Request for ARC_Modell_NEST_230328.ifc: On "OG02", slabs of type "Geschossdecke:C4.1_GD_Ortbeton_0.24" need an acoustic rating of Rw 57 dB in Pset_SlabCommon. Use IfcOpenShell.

First a look at what the model holds.

```python
import ifcopenshell
import ifcopenshell.util.element

model = ifcopenshell.open("ARC_Modell_NEST_230328.ifc")
print(model.schema)
storey = next(s for s in model.by_type("IfcBuildingStorey") if s.Name == "OG02")
slabs = [e for e in ifcopenshell.util.element.get_decomposition(storey) if e.is_a("IfcSlab")]
seen = {}
for e in slabs:
    element_type = ifcopenshell.util.element.get_type(e)
    key = (element_type.Name if element_type != e and element_type else None, ifcopenshell.util.element.get_pset(e, "Pset_SlabCommon", "AcousticRating"))
    seen[key] = seen.get(key, 0) + 1
for (name, value), count in sorted(seen.items(), key=str):
    print(count, "x", name, "|", value)
```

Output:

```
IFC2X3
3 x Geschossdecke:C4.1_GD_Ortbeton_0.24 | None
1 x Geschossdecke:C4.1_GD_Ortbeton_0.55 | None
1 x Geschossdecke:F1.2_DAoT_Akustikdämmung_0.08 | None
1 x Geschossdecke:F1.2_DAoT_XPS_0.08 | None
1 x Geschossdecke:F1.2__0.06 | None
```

```python
import ifcopenshell
import ifcopenshell.api.pset
import ifcopenshell.util.element

model = ifcopenshell.open("ARC_Modell_NEST_230328.ifc")

storey = next(s for s in model.by_type("IfcBuildingStorey") if s.Name == "OG02")
slabs = [e for e in ifcopenshell.util.element.get_decomposition(storey) if e.is_a("IfcSlab")]

count = 0
for e in slabs:
    element_type = ifcopenshell.util.element.get_type(e)
    if element_type in (None, e) or element_type.Name != "Geschossdecke:C4.1_GD_Ortbeton_0.24":
        continue
    # add_pset returns the element's existing set when there is one.
    pset = ifcopenshell.api.pset.add_pset(model, product=e, name="Pset_SlabCommon")
    ifcopenshell.api.pset.edit_pset(model, pset=pset, properties={"AcousticRating": "Rw 57 dB"})
    count += 1

print(count, "slabs updated")

model.write("ARC_Modell_NEST_230328_updated.ifc")
```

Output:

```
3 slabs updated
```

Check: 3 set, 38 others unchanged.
